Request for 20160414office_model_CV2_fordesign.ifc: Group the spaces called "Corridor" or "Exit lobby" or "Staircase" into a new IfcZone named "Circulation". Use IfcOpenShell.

First a look at what the model holds.

```python
import ifcopenshell

model = ifcopenshell.open("20160414office_model_CV2_fordesign.ifc")
print(model.schema)
seen = {}
for space in model.by_type("IfcSpace"):
    seen[space.LongName] = seen.get(space.LongName, 0) + 1
for name, count in sorted(seen.items(), key=str):
    print(count, "x", name)
print("zones:", [z.Name for z in model.by_type("IfcZone")][:20])
```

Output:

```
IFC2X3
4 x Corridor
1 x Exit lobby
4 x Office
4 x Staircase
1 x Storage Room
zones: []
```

```python
import ifcopenshell
import ifcopenshell.api.group
import ifcopenshell.api.root

model = ifcopenshell.open("20160414office_model_CV2_fordesign.ifc")

names = {"Corridor", "Exit lobby", "Staircase"}
spaces = [s for s in model.by_type("IfcSpace") if s.LongName in names]

zone = ifcopenshell.api.root.create_entity(model, ifc_class="IfcZone", name="Circulation")
ifcopenshell.api.group.assign_group(model, products=spaces, group=zone)
print(len(spaces), "spaces in", zone.Name)

model.write("20160414office_model_CV2_fordesign-out.ifc")
```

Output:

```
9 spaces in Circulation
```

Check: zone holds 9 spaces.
